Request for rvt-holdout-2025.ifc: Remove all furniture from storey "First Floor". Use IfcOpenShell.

First a look at what the model holds.

```python
import ifcopenshell
import ifcopenshell.util.element

model = ifcopenshell.open("rvt-holdout-2025.ifc")
print(model.schema)
storey = next(s for s in model.by_type("IfcBuildingStorey") if s.Name == "First Floor")
furniture = [e for e in ifcopenshell.util.element.get_decomposition(storey) if e.is_a("IfcFurnishingElement")]
seen = {}
for e in furniture:
    element_type = ifcopenshell.util.element.get_type(e)
    name = element_type.Name if element_type not in (None, e) else None
    seen[name] = seen.get(name, 0) + 1
for name, count in sorted(seen.items(), key=str):
    print(count, "x", name)
```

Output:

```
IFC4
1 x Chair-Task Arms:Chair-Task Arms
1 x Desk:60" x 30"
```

```python
import ifcopenshell
import ifcopenshell.api.root
import ifcopenshell.util.element

model = ifcopenshell.open("rvt-holdout-2025.ifc")

storey = next(s for s in model.by_type("IfcBuildingStorey") if s.Name == "First Floor")
furniture = [e for e in ifcopenshell.util.element.get_decomposition(storey) if e.is_a("IfcFurnishingElement")]

for e in furniture:
    ifcopenshell.api.root.remove_product(model, product=e)
print(len(furniture), "removed")

model.write("rvt-holdout-2025-out.ifc")
```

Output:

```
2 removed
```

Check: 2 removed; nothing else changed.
